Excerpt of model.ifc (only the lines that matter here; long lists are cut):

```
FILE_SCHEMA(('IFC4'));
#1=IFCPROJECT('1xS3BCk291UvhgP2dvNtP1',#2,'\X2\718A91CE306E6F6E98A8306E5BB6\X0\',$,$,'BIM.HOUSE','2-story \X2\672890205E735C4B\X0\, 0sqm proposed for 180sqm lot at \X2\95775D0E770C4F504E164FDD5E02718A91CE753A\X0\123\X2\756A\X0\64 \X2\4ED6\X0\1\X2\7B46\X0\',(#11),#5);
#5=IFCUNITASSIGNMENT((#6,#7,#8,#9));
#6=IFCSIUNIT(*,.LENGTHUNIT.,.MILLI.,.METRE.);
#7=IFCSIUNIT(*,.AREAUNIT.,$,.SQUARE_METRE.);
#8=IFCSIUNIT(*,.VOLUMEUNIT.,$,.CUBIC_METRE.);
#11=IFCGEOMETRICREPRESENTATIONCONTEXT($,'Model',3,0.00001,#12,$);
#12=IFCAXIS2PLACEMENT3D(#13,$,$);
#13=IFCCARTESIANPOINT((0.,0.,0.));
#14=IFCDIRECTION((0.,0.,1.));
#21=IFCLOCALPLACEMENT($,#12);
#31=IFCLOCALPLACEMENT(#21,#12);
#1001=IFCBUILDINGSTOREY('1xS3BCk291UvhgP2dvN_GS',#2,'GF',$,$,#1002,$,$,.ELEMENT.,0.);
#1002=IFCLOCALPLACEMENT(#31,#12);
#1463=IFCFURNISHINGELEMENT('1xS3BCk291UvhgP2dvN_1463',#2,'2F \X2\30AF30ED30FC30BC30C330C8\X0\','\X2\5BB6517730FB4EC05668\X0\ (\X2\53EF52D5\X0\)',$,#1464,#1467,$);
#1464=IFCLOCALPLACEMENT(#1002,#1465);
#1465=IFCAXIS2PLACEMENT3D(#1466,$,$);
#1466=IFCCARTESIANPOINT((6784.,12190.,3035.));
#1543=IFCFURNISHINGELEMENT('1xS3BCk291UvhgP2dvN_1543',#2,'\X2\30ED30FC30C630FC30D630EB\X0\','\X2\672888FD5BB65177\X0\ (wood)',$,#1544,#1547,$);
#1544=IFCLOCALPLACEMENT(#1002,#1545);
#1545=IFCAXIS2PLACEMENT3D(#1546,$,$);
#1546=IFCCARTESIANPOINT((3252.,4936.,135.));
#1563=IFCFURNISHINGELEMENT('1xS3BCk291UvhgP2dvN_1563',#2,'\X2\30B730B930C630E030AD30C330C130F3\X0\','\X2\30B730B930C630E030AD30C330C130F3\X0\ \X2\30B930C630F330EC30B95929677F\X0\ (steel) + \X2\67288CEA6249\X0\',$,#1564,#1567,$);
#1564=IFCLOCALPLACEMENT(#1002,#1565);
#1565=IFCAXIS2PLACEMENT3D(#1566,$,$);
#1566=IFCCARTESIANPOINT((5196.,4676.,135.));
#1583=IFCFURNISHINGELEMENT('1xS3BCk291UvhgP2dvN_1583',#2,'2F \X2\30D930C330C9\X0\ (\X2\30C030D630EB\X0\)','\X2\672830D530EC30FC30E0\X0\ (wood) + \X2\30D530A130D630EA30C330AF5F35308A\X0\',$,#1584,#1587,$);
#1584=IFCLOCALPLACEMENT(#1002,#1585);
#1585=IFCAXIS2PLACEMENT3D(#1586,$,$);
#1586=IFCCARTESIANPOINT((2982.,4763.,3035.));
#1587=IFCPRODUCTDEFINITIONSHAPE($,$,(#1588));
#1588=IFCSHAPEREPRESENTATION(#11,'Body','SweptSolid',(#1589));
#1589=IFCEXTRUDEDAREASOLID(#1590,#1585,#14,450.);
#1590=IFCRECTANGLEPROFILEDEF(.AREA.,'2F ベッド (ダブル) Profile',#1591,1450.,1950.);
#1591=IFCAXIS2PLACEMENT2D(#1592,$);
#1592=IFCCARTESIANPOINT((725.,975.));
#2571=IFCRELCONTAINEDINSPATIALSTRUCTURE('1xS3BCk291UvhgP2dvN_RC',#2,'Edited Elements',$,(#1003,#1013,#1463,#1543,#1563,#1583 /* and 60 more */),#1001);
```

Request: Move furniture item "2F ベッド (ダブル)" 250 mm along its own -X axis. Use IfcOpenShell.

```python
import ifcopenshell
import ifcopenshell.api.geometry
import ifcopenshell.util.placement
import ifcopenshell.util.unit

model = ifcopenshell.open("model.ifc")
unit_scale = ifcopenshell.util.unit.calculate_unit_scale(model)

item = model.by_id(1583)
matrix = ifcopenshell.util.placement.get_local_placement(item.ObjectPlacement)
matrix[:3, 3] -= matrix[:3, 0] * 0.25 / unit_scale
ifcopenshell.api.geometry.edit_object_placement(model, product=item, matrix=matrix, is_si=False)

print(ifcopenshell.util.placement.get_local_placement(item.ObjectPlacement).round(3) + 0.0)

model.write("model_edited.ifc")
```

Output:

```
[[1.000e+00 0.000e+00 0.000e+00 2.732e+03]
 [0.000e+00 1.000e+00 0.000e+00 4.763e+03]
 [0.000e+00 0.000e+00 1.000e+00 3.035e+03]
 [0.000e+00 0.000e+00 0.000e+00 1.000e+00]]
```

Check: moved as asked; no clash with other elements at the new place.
